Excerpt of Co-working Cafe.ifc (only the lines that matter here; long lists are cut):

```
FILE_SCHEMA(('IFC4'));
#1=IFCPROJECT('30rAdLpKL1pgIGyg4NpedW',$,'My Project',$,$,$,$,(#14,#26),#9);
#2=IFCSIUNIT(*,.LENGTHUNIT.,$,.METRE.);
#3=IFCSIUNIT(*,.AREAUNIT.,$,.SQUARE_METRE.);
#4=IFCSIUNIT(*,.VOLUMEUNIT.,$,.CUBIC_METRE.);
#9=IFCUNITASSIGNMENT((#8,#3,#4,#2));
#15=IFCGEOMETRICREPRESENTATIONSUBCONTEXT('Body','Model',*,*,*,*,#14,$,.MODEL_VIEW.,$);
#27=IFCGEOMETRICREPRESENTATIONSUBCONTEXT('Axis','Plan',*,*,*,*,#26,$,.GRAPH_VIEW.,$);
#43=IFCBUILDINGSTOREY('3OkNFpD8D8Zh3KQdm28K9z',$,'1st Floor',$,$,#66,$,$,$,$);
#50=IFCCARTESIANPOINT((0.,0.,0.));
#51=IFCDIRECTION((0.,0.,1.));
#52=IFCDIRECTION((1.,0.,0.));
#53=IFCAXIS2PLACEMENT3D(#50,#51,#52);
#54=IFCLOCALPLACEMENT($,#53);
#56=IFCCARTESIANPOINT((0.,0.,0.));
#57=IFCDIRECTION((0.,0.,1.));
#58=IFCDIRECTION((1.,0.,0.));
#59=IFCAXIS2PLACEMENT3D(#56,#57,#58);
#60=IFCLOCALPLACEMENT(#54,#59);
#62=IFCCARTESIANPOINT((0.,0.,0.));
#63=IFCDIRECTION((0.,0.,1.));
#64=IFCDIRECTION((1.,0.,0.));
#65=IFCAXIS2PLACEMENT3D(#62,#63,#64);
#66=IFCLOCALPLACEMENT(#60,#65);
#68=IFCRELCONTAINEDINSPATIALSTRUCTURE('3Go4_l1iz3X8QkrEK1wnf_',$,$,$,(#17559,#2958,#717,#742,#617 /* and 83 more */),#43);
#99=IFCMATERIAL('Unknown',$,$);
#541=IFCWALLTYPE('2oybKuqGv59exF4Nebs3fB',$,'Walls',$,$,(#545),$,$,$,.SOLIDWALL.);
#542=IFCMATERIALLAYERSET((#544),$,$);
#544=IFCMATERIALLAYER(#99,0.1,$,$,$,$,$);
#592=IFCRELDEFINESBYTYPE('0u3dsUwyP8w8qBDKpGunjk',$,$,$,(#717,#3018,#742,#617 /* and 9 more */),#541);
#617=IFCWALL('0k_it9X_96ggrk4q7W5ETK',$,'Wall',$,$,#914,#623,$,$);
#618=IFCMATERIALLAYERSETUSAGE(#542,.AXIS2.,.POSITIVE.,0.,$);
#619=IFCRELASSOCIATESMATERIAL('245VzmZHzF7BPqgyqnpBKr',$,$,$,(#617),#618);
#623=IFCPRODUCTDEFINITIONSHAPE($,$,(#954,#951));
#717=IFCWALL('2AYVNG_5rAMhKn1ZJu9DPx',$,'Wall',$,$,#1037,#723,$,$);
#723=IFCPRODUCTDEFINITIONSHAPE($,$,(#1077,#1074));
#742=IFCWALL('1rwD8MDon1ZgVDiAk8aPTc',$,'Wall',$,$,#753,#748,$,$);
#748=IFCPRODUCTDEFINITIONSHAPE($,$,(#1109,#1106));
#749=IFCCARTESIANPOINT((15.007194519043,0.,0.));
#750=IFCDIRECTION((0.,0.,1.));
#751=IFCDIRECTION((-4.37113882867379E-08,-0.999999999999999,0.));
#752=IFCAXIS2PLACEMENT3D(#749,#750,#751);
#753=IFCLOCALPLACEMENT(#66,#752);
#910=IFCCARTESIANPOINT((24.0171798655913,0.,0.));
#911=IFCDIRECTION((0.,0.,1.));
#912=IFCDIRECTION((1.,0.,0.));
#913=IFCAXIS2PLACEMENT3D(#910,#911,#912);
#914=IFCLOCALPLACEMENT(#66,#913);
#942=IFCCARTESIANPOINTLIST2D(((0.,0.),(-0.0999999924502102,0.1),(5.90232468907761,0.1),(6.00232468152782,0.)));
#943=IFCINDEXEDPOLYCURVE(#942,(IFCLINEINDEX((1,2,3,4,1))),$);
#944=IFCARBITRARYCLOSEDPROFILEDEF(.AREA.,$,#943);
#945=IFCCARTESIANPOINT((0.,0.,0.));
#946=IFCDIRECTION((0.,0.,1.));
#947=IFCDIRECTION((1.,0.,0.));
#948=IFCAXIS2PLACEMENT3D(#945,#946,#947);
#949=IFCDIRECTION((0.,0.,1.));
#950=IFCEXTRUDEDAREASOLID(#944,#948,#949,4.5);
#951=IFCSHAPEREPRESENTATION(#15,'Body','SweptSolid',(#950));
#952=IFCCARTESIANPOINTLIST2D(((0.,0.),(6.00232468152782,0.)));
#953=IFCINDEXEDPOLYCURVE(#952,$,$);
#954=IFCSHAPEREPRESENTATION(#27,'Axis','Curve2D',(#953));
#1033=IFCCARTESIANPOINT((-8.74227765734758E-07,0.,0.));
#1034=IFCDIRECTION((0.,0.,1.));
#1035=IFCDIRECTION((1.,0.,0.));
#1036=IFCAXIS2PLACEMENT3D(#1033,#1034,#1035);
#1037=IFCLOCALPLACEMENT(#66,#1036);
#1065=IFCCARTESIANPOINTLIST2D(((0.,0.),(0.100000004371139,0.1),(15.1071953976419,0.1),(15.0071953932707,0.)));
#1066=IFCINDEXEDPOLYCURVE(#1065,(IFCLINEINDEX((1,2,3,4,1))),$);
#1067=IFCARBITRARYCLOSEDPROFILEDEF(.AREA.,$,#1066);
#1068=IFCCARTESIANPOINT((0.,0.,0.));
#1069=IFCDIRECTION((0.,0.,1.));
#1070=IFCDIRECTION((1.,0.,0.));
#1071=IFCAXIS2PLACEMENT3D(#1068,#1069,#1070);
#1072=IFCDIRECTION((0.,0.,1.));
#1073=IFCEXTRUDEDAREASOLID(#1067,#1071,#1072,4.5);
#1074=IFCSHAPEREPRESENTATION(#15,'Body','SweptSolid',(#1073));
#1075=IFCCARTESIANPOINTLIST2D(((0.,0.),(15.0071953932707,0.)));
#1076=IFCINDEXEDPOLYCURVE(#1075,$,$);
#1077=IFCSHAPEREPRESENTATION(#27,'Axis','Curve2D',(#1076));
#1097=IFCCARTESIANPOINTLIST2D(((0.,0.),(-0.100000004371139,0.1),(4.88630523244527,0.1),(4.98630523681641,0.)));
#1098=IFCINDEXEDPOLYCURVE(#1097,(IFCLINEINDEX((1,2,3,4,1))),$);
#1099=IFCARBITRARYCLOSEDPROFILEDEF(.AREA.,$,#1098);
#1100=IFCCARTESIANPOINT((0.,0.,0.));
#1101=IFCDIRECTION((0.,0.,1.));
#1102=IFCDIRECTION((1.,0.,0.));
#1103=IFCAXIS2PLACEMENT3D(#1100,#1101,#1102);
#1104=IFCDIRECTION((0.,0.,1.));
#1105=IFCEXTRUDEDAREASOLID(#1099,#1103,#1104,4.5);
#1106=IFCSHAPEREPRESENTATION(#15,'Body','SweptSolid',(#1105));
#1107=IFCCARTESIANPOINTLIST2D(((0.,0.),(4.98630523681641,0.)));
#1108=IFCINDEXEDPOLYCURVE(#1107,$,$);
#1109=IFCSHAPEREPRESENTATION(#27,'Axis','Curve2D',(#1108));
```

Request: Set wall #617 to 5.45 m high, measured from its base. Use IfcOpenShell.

```python
import ifcopenshell
import ifcopenshell.geom
import ifcopenshell.util.representation
import ifcopenshell.util.shape
import ifcopenshell.util.unit

model = ifcopenshell.open("Co-working Cafe.ifc")
unit_scale = ifcopenshell.util.unit.calculate_unit_scale(model)
settings = ifcopenshell.geom.settings()


def volume(element):
    """Net volume in cubic metres, openings subtracted."""
    shape = ifcopenshell.geom.create_shape(settings, element)
    return ifcopenshell.util.shape.get_volume(shape.geometry)


wall = model.by_guid("0k_it9X_96ggrk4q7W5ETK")
before = volume(wall)

body = ifcopenshell.util.representation.get_representation(wall, "Model", "Body")
solid = body.Items[0]
old_height = solid.Depth
solid.Depth = 5.45 / unit_scale
after = volume(wall)

print(f"height {old_height:g} -> {solid.Depth:g}, volume {before:.3f} -> {after:.3f} m3")

model.write("Co-working Cafe_v2.ifc")
```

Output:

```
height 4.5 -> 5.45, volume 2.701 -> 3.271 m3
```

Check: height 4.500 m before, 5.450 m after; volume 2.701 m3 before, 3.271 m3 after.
